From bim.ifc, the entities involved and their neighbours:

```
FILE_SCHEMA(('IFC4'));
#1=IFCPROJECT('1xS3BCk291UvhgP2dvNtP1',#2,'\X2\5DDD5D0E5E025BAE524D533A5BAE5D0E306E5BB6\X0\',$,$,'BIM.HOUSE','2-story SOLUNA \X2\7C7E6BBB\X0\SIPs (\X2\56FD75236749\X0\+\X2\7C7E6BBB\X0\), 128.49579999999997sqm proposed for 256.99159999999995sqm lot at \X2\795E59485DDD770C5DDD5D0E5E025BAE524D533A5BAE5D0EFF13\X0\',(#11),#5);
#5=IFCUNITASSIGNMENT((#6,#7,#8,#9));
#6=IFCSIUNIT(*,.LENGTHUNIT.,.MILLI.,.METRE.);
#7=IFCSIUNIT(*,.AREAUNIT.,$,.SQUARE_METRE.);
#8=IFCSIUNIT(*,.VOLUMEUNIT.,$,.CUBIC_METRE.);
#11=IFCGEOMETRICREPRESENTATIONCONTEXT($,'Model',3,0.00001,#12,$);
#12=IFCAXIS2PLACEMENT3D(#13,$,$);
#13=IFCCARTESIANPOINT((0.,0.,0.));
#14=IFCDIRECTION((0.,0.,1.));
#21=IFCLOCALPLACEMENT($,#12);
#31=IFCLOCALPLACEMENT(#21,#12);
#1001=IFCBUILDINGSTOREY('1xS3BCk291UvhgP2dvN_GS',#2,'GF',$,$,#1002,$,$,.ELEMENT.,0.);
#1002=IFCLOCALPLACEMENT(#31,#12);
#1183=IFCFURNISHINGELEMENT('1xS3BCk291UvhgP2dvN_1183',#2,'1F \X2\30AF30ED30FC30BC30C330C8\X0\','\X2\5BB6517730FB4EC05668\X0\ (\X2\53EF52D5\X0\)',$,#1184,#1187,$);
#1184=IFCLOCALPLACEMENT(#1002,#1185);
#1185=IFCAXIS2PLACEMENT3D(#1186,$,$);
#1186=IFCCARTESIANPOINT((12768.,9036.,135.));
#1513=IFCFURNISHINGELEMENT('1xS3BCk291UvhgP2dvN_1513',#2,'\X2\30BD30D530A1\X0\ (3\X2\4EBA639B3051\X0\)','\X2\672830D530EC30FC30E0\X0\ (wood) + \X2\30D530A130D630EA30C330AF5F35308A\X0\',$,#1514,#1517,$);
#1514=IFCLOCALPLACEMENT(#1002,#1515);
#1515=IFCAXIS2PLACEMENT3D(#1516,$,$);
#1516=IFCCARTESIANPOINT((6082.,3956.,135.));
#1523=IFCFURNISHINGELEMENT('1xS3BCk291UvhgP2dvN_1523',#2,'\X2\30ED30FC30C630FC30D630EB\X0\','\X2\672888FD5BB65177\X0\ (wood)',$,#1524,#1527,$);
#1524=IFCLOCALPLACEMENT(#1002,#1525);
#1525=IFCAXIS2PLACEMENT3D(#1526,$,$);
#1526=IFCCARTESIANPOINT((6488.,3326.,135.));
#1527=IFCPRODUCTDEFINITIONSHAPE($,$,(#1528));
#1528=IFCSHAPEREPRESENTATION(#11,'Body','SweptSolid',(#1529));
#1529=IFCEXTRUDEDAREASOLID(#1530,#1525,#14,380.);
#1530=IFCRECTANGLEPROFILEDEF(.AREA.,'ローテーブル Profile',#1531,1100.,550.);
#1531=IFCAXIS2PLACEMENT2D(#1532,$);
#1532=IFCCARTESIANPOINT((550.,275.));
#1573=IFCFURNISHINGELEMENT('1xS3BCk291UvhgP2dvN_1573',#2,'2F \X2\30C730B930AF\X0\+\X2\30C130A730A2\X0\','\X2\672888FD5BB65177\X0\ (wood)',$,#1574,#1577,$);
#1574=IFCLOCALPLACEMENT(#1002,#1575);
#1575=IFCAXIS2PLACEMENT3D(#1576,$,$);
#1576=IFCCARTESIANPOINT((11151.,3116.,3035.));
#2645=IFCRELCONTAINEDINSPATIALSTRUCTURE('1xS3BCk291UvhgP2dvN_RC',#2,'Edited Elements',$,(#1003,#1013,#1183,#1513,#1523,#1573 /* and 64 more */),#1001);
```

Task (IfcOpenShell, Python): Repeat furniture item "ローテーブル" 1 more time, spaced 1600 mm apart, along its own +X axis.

```python
import ifcopenshell
import ifcopenshell.api.geometry
import ifcopenshell.api.root
import ifcopenshell.util.element
import ifcopenshell.util.placement
import ifcopenshell.util.unit

model = ifcopenshell.open("bim.ifc")
unit_scale = ifcopenshell.util.unit.calculate_unit_scale(model)


def reuse_history(source, copy):
    """copy_class also copies each property set's owner history, people and application; keep the originals."""
    for rel in copy.IsDefinedBy:
        if rel.is_a("IfcRelDefinesByProperties") and (history := rel.RelatingPropertyDefinition.OwnerHistory):
            rel.RelatingPropertyDefinition.OwnerHistory = source.OwnerHistory
            ifcopenshell.util.element.remove_deep2(model, history)


source = model.by_id(1523)
base = ifcopenshell.util.placement.get_local_placement(source.ObjectPlacement)
step = base[:3, 0] * 1.6 / unit_scale

for i in range(1, 2):
    copy = ifcopenshell.api.root.copy_class(model, product=source)
    copy.Representation = ifcopenshell.util.element.copy_deep(
        model, source.Representation, exclude=["IfcGeometricRepresentationContext", "IfcRepresentationMap"]
    )
    reuse_history(source, copy)
    matrix = base.copy()
    matrix[:3, 3] += i * step
    print("added at", matrix[:3, 3].round(3) + 0.0)
    ifcopenshell.api.geometry.edit_object_placement(model, product=copy, matrix=matrix, is_si=False)

model.write("bim_v2.ifc")
```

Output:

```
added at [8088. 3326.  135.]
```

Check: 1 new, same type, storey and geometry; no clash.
